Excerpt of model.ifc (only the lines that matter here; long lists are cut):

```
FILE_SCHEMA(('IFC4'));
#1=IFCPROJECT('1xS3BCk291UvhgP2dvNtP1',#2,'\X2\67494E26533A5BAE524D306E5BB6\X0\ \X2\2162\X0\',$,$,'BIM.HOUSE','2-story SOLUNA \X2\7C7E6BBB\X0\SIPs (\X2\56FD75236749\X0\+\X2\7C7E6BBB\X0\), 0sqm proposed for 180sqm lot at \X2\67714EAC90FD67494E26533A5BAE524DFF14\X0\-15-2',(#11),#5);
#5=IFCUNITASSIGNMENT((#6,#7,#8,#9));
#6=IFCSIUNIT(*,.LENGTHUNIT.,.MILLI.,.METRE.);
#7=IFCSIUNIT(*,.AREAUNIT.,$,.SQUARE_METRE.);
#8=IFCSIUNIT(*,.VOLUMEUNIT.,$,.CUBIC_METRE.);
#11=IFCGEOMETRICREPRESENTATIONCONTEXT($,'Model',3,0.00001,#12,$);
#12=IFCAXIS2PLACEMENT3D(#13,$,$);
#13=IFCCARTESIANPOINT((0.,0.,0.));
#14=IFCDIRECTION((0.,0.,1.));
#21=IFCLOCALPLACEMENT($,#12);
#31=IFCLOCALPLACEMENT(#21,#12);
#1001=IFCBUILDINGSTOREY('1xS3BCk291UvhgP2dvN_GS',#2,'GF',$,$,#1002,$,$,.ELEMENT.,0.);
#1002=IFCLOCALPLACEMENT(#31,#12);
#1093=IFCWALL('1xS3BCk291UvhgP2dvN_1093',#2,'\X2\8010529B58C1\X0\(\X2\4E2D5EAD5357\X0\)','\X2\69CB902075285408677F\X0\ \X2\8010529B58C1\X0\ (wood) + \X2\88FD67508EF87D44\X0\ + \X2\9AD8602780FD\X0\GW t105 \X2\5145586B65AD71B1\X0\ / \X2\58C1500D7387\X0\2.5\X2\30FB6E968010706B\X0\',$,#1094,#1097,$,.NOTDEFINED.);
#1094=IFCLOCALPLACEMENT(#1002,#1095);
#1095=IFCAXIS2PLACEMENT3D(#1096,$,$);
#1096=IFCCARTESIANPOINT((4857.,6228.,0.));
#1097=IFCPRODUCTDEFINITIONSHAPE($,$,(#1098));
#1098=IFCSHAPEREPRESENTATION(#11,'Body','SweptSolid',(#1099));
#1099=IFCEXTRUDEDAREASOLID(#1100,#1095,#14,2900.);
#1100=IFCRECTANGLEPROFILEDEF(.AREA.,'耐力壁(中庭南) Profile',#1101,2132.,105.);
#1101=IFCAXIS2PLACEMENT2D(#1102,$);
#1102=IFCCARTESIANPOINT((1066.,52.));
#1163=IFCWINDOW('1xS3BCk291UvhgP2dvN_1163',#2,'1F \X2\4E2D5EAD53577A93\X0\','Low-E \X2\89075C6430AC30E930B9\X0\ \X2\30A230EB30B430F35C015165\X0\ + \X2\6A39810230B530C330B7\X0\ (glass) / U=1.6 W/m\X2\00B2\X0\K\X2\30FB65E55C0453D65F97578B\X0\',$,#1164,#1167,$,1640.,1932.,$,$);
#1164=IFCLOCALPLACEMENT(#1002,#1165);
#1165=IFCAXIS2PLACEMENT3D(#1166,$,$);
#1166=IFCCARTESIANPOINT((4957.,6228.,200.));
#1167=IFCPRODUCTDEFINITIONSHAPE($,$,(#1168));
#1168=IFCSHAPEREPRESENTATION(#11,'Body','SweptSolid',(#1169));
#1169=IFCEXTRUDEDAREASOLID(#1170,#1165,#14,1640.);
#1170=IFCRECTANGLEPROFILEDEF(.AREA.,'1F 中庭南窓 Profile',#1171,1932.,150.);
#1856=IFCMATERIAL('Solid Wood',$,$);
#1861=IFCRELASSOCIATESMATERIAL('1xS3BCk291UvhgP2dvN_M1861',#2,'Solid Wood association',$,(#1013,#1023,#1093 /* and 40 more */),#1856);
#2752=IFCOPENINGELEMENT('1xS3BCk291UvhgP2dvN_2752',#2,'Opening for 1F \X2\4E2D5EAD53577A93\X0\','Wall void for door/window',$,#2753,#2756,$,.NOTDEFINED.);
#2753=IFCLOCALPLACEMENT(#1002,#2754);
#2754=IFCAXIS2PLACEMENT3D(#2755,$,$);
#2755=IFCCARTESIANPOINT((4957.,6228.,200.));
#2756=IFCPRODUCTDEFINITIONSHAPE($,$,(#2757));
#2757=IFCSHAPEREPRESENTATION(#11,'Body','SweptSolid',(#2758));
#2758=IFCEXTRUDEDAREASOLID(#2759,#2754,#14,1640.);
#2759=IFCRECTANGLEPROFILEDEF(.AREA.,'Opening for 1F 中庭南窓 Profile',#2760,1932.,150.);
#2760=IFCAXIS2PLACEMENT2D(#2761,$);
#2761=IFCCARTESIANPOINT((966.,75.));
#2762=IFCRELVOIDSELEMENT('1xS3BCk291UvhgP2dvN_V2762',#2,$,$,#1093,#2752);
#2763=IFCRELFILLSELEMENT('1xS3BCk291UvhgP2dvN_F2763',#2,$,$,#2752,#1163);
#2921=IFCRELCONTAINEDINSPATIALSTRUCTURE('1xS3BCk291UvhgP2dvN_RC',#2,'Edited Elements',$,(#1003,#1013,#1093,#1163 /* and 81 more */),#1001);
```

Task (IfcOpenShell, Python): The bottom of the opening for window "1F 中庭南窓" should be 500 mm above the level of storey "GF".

```python
import numpy as np
import ifcopenshell
import ifcopenshell.api.geometry
import ifcopenshell.geom
import ifcopenshell.util.element
import ifcopenshell.util.placement
import ifcopenshell.util.shape
import ifcopenshell.util.unit

model = ifcopenshell.open("model.ifc")
unit_scale = ifcopenshell.util.unit.calculate_unit_scale(model)

window = model.by_guid("1xS3BCk291UvhgP2dvN_1163")
opening = window.FillsVoids[0].RelatingOpeningElement
storey = ifcopenshell.util.element.get_container(window, ifc_class="IfcBuildingStorey")
level = ifcopenshell.util.placement.get_local_placement(storey.ObjectPlacement)[2, 3]

# The opening's origin need not be at the sill, so measure its lowest point.
shape = ifcopenshell.geom.create_shape(ifcopenshell.geom.settings(), opening)
bottom = ifcopenshell.util.shape.get_shape_bottom_elevation(shape, shape.geometry) / unit_scale
dz = level + 0.5 / unit_scale - bottom

shift = np.array([0.0, 0.0, dz])
# The window is not placed relative to its opening, so move both.
for product in (opening, window):
    matrix = ifcopenshell.util.placement.get_local_placement(product.ObjectPlacement)
    matrix[:3, 3] += shift
    ifcopenshell.api.geometry.edit_object_placement(model, product=product, matrix=matrix, is_si=False)

print(f"moved by {dz * unit_scale:+.3f} m")

model.write("model_rev.ifc")
```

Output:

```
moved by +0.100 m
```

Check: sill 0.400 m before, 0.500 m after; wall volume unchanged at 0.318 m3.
